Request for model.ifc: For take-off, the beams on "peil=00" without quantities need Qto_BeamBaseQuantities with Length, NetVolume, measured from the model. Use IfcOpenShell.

First a look at what the model holds.

```python
import ifcopenshell
import ifcopenshell.util.element
import ifcopenshell.util.unit

model = ifcopenshell.open("model.ifc")
print(model.schema)
for unit_type in ("LENGTHUNIT", "AREAUNIT", "VOLUMEUNIT"):
    print(unit_type, ifcopenshell.util.unit.calculate_unit_scale(model, unit_type))
storey = next(s for s in model.by_type("IfcBuildingStorey") if s.Name == "peil=00")
beams = [e for e in ifcopenshell.util.element.get_decomposition(storey) if e.is_a("IfcBeam")]
for e in sorted(beams, key=lambda e: e.id()):
    print(e.id(), e.is_a(), e.Name, list(ifcopenshell.util.element.get_psets(e, qtos_only=True)), sep=" | ")
```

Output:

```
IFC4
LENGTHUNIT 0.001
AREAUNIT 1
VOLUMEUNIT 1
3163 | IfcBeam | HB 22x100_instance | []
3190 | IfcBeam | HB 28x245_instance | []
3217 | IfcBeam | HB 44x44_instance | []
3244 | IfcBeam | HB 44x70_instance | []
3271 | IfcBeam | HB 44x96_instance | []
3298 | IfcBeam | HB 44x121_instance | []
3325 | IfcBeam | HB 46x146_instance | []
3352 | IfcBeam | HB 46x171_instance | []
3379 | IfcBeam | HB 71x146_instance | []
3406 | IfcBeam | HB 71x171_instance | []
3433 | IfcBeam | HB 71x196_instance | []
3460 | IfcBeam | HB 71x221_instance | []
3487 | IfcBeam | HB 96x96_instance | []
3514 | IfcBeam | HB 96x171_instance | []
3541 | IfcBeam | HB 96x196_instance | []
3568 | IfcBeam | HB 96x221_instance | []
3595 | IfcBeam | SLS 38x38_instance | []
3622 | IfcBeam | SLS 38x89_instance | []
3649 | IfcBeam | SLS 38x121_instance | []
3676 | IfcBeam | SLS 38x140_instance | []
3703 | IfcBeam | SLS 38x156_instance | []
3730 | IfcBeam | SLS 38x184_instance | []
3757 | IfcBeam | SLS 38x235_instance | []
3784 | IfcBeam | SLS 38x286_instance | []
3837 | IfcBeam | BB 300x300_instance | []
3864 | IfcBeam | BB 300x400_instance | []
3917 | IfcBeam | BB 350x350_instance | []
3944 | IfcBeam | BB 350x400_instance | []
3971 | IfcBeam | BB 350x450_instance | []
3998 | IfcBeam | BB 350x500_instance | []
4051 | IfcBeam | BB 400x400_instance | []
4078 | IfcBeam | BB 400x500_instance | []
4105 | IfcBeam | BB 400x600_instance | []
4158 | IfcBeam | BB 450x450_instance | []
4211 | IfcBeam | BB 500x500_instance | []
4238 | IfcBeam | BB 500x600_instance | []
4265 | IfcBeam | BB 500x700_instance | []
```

```python
import ifcopenshell
import ifcopenshell.api.pset
import ifcopenshell.geom
import ifcopenshell.util.element
import ifcopenshell.util.shape
import ifcopenshell.util.unit

model = ifcopenshell.open("model.ifc")
unit_scale = ifcopenshell.util.unit.calculate_unit_scale(model)
volume_scale = ifcopenshell.util.unit.calculate_unit_scale(model, "VOLUMEUNIT")
settings = ifcopenshell.geom.settings()

storey = next(s for s in model.by_type("IfcBuildingStorey") if s.Name == "peil=00")
beams = [e for e in ifcopenshell.util.element.get_decomposition(storey) if e.is_a("IfcBeam")]

for e in sorted(beams, key=lambda e: e.id()):
    if ifcopenshell.util.element.get_psets(e, qtos_only=True, should_inherit=False):
        continue
    # Geometry comes back in metres, in the element's own axes.
    shape = ifcopenshell.geom.create_shape(settings, e)
    values = {
        "Length": ifcopenshell.util.shape.get_max_xyz(shape.geometry) / unit_scale,
        "NetVolume": ifcopenshell.util.shape.get_volume(shape.geometry) / volume_scale,
    }
    qto = ifcopenshell.api.pset.add_qto(model, product=e, name="Qto_BeamBaseQuantities")
    ifcopenshell.api.pset.edit_qto(model, qto=qto, properties=values)
    print(e.id(), {k: round(v, 3) for k, v in values.items()})

model.write("model_v2.ifc")
```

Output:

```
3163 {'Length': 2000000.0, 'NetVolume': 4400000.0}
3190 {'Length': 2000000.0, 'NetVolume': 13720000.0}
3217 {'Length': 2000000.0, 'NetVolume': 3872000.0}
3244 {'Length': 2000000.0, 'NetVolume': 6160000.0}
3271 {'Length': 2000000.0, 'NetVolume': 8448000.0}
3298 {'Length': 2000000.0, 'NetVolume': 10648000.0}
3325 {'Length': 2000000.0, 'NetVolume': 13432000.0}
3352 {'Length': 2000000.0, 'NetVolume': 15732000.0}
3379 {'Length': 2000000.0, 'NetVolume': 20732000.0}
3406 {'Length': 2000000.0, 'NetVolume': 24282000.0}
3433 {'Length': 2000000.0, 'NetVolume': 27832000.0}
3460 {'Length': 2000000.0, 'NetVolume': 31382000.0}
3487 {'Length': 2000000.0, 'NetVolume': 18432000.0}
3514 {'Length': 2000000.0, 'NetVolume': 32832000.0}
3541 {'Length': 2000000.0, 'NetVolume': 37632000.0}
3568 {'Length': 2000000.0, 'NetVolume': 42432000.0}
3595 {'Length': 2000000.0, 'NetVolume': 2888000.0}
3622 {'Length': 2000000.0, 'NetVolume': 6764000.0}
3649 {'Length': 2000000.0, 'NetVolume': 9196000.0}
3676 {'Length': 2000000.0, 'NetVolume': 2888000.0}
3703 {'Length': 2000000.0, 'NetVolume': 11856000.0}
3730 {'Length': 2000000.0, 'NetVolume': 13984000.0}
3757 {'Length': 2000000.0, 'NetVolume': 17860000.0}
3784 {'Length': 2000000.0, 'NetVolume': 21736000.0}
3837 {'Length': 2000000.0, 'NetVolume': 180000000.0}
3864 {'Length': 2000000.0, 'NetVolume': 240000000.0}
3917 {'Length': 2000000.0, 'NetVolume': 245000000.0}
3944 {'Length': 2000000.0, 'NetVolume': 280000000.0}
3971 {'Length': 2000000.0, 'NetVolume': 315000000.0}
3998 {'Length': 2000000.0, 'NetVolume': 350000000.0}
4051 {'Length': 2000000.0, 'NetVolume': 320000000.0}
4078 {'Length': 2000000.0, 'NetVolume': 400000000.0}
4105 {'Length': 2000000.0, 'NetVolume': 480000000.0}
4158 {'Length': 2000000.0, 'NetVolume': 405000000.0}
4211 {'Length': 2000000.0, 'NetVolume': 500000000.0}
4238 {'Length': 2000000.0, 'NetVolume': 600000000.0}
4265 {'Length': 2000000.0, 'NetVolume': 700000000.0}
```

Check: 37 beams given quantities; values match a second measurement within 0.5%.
